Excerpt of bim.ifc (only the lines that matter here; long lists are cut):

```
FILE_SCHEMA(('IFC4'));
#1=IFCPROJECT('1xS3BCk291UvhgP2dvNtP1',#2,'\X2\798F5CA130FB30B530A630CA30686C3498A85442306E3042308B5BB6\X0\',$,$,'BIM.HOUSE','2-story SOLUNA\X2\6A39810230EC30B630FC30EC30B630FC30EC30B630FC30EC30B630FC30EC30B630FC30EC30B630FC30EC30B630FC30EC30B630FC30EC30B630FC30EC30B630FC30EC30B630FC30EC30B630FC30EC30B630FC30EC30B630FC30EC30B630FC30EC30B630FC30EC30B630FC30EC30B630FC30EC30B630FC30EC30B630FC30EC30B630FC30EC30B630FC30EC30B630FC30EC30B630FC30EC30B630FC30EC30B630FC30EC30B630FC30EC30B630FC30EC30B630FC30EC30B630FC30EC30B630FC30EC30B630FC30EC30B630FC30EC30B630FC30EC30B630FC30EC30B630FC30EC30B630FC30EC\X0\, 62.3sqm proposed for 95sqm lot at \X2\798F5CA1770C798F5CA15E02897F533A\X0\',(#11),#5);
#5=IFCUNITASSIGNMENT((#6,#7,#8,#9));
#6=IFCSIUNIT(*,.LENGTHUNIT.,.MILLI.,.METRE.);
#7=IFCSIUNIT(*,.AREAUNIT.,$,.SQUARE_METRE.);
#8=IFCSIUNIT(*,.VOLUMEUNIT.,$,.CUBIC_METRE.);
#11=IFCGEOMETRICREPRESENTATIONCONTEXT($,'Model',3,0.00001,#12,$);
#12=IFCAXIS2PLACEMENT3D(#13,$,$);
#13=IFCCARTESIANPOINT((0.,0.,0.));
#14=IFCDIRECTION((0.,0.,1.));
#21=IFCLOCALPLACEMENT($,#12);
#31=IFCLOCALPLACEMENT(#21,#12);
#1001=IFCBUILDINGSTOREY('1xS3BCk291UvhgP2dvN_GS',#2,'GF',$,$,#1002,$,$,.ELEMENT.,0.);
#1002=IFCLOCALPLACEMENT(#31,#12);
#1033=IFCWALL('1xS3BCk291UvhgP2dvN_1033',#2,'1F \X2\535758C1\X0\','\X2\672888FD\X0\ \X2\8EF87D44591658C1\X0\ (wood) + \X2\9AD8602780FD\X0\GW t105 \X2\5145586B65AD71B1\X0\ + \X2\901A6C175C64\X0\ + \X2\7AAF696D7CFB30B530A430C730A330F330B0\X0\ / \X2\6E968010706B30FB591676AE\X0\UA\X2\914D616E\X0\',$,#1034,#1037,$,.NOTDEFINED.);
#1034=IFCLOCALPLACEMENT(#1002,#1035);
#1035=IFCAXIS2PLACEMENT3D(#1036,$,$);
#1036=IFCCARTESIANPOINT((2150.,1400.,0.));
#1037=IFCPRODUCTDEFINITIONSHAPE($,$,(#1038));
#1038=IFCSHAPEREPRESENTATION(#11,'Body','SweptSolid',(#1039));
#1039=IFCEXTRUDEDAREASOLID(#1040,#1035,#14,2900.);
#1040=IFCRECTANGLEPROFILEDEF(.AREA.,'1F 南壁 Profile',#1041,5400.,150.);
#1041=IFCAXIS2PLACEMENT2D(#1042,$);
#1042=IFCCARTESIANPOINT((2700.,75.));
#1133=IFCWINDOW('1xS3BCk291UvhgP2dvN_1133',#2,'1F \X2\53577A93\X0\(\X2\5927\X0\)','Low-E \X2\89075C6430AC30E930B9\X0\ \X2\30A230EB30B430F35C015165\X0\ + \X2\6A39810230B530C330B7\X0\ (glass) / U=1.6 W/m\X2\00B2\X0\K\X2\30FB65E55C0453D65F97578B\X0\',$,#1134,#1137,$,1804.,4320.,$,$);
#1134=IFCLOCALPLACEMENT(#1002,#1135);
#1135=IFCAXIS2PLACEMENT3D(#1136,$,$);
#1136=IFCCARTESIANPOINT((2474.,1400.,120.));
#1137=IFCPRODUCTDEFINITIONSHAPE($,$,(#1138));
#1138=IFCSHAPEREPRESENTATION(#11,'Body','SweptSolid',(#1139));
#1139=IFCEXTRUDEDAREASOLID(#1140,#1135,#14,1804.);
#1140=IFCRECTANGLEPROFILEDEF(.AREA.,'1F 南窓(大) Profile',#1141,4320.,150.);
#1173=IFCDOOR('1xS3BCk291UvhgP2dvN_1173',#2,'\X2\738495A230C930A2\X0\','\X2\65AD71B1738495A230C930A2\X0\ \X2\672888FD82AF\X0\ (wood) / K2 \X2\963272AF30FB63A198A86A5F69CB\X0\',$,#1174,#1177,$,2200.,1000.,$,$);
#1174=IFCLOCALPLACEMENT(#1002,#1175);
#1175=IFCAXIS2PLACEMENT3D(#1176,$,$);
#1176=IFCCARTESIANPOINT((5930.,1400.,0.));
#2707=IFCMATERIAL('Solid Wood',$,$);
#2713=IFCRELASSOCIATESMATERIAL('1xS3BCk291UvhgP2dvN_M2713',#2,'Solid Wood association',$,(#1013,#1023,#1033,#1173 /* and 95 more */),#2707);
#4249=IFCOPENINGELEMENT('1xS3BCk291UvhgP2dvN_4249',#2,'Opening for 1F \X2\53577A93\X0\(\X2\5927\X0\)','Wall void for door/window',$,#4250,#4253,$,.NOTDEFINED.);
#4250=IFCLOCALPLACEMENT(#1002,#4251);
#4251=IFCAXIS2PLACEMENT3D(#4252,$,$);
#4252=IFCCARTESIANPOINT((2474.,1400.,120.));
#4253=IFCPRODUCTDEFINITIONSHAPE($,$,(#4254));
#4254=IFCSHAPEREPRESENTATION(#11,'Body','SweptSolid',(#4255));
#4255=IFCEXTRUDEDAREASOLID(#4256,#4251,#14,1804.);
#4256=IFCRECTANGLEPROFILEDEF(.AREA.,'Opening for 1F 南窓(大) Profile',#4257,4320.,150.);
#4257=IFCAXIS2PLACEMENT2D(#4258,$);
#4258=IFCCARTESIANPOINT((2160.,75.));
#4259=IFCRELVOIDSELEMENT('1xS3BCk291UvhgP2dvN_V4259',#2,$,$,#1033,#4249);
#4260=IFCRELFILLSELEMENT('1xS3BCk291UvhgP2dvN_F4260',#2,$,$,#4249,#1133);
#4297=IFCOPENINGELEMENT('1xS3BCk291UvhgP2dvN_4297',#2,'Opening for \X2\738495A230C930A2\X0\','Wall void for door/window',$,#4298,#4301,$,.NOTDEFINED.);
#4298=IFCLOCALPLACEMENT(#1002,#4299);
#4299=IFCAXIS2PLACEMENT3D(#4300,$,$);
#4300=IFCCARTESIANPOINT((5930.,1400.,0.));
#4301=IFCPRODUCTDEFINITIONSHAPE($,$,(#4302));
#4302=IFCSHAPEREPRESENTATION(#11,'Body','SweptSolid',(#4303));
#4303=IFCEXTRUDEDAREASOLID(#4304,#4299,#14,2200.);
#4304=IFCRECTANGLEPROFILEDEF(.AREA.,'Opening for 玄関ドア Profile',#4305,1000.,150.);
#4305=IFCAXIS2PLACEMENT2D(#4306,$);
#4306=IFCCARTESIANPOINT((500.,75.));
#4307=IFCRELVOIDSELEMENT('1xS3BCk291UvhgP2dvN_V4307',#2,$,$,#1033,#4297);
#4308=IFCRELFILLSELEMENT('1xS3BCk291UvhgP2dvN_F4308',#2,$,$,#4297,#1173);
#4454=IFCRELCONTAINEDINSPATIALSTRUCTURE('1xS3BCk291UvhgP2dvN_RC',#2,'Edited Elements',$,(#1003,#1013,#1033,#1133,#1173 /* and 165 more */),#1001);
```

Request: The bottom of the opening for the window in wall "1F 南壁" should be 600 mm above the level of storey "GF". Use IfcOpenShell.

```python
import numpy as np
import ifcopenshell
import ifcopenshell.api.geometry
import ifcopenshell.geom
import ifcopenshell.util.element
import ifcopenshell.util.placement
import ifcopenshell.util.shape
import ifcopenshell.util.unit

model = ifcopenshell.open("bim.ifc")
unit_scale = ifcopenshell.util.unit.calculate_unit_scale(model)

window = model.by_guid("1xS3BCk291UvhgP2dvN_1133")
opening = window.FillsVoids[0].RelatingOpeningElement
storey = ifcopenshell.util.element.get_container(window, ifc_class="IfcBuildingStorey")
level = ifcopenshell.util.placement.get_local_placement(storey.ObjectPlacement)[2, 3]

# The opening's origin need not be at the sill, so measure its lowest point.
shape = ifcopenshell.geom.create_shape(ifcopenshell.geom.settings(), opening)
bottom = ifcopenshell.util.shape.get_shape_bottom_elevation(shape, shape.geometry) / unit_scale
dz = level + 600.0 - bottom

shift = np.array([0.0, 0.0, dz])
# The window is not placed relative to its opening, so move both.
for product in (opening, window):
    matrix = ifcopenshell.util.placement.get_local_placement(product.ObjectPlacement)
    matrix[:3, 3] += shift
    ifcopenshell.api.geometry.edit_object_placement(model, product=product, matrix=matrix, is_si=False)

print(f"moved by {dz * unit_scale:+.3f} m")

model.write("bim-out.ifc")
```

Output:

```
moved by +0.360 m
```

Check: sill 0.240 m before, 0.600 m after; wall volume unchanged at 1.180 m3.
